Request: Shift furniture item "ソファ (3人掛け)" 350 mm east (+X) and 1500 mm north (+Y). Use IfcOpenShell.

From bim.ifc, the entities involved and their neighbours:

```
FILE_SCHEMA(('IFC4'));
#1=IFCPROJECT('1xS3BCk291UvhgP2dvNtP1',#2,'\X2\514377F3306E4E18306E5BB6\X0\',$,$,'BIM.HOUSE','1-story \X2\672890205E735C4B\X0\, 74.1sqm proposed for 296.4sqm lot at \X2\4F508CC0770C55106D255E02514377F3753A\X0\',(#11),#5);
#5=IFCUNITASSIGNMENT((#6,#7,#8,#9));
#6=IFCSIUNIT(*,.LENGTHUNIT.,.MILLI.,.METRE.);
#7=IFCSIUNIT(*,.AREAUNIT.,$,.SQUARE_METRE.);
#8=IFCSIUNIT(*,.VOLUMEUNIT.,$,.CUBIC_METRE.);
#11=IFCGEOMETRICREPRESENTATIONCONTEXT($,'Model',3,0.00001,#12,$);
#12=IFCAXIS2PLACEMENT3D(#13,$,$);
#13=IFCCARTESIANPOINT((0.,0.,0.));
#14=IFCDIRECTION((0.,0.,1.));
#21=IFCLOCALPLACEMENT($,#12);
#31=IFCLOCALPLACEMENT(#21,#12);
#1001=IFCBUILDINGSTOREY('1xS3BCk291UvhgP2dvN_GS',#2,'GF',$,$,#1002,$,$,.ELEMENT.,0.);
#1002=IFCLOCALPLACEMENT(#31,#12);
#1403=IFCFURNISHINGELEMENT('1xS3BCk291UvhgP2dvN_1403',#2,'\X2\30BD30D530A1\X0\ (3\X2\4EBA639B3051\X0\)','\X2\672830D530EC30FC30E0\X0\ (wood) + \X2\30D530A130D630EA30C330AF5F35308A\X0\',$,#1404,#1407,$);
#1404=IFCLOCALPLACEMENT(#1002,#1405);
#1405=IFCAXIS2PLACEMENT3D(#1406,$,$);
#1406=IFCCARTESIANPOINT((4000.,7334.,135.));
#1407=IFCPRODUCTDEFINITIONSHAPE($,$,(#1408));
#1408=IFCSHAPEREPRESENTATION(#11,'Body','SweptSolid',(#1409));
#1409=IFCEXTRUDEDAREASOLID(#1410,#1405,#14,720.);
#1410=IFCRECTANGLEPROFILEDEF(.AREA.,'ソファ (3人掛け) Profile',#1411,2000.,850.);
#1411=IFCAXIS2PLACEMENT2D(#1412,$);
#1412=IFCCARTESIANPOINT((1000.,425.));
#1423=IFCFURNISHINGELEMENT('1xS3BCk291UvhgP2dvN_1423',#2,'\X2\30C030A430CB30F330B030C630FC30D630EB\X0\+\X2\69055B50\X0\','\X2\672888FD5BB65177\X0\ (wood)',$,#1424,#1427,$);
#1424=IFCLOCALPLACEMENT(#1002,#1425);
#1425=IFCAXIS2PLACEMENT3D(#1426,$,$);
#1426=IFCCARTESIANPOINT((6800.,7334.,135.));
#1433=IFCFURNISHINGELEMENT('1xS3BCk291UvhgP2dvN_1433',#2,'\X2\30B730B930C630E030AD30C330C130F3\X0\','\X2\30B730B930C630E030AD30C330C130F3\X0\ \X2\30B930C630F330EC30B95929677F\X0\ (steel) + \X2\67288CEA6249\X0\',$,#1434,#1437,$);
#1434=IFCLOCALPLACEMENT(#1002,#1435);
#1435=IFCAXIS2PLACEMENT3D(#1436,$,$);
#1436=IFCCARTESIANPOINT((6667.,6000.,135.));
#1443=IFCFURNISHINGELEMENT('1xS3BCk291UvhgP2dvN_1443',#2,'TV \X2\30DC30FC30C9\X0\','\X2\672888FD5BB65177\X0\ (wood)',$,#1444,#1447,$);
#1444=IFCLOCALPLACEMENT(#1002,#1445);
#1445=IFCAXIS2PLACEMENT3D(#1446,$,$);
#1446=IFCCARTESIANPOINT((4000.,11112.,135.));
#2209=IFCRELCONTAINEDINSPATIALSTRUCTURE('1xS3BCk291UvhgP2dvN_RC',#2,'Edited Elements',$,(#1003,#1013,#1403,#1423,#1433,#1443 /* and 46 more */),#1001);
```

```python
import ifcopenshell
import ifcopenshell.api.geometry
import ifcopenshell.util.placement

model = ifcopenshell.open("bim.ifc")

item = model.by_guid("1xS3BCk291UvhgP2dvN_1403")
matrix = ifcopenshell.util.placement.get_local_placement(item.ObjectPlacement)
matrix[0, 3] += 350.0
matrix[1, 3] += 1500.0
ifcopenshell.api.geometry.edit_object_placement(model, product=item, matrix=matrix, is_si=False)

print(ifcopenshell.util.placement.get_local_placement(item.ObjectPlacement).round(3) + 0.0)

model.write("bim_edited.ifc")
```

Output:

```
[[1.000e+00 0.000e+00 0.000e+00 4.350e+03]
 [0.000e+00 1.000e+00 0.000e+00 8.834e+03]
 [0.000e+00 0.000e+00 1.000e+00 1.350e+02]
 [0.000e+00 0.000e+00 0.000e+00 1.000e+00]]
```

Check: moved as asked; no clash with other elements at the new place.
